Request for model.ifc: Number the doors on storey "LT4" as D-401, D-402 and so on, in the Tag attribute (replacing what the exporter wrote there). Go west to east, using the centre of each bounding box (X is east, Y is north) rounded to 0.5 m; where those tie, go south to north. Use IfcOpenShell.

First a look at what the model holds.

```python
import ifcopenshell
import ifcopenshell.util.element
import ifcopenshell.util.placement

model = ifcopenshell.open("model.ifc")
print(model.schema)
storey = next(s for s in model.by_type("IfcBuildingStorey") if s.Name == "LT4")
doors = [e for e in ifcopenshell.util.element.get_decomposition(storey) if e.is_a("IfcDoor")]
for e in sorted(doors, key=lambda e: e.id()):
    origin = ifcopenshell.util.placement.get_local_placement(e.ObjectPlacement)[:3, 3]
    print(e.id(), e.Tag, e.Name, origin.round(2) + 0.0, sep=" | ")
```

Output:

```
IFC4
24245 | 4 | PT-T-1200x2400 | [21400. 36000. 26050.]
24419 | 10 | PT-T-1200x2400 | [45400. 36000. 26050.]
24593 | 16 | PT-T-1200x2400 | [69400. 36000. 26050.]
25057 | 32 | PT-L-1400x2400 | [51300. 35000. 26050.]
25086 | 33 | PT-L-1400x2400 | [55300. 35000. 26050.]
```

```python
import ifcopenshell
import ifcopenshell.geom
import ifcopenshell.util.element
import ifcopenshell.util.shape

model = ifcopenshell.open("model.ifc")
settings = ifcopenshell.geom.settings()
settings.set("use-world-coords", True)


def centre(element):
    shape = ifcopenshell.geom.create_shape(settings, element)
    return ifcopenshell.util.shape.get_bbox_centroid(shape.geometry)


storey = next(s for s in model.by_type("IfcBuildingStorey") if s.Name == "LT4")
doors = [e for e in ifcopenshell.util.element.get_decomposition(storey) if e.is_a("IfcDoor")]

# Insertion points can sit at a corner or the storey origin, so sort by the geometry (in metres).
centres = {e: centre(e) for e in doors}
doors.sort(key=lambda e: (round(centres[e][0] / 0.5), centres[e][1]))

for i, e in enumerate(doors, start=1):
    number = f"D-4{i:02d}"
    e.Tag = number
    print(e.id(), number)

model.write("model_rev.ifc")
```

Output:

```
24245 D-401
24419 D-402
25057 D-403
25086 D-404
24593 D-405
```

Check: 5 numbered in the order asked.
